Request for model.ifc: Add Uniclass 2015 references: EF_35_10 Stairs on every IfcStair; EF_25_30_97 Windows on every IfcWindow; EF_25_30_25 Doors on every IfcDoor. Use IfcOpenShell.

First a look at what the model holds.

```python
import ifcopenshell

model = ifcopenshell.open("model.ifc")
print(model.schema)
print("classifications:", [c.Name for c in model.by_type("IfcClassification")])
for ifc_class in ("IfcDoor", "IfcRoof", "IfcStair", "IfcWall", "IfcWindow"):
    print(ifc_class, len(model.by_type(ifc_class)))
```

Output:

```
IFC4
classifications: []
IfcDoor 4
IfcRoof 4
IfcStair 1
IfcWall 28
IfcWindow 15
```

```python
import ifcopenshell
import ifcopenshell.api.classification

model = ifcopenshell.open("model.ifc")

system = ifcopenshell.api.classification.add_classification(model, classification="Uniclass 2015")

codes = {
    "IfcStair": ("EF_35_10", "Stairs"),
    "IfcWindow": ("EF_25_30_97", "Windows"),
    "IfcDoor": ("EF_25_30_25", "Doors"),
}
for ifc_class, (code, name) in codes.items():
    products = model.by_type(ifc_class)
    ifcopenshell.api.classification.add_reference(
        model, products=products, classification=system, identification=code, name=name
    )
    print(code, len(products))

model.write("model_rev.ifc")
```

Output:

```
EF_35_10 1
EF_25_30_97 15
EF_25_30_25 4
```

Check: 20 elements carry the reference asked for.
